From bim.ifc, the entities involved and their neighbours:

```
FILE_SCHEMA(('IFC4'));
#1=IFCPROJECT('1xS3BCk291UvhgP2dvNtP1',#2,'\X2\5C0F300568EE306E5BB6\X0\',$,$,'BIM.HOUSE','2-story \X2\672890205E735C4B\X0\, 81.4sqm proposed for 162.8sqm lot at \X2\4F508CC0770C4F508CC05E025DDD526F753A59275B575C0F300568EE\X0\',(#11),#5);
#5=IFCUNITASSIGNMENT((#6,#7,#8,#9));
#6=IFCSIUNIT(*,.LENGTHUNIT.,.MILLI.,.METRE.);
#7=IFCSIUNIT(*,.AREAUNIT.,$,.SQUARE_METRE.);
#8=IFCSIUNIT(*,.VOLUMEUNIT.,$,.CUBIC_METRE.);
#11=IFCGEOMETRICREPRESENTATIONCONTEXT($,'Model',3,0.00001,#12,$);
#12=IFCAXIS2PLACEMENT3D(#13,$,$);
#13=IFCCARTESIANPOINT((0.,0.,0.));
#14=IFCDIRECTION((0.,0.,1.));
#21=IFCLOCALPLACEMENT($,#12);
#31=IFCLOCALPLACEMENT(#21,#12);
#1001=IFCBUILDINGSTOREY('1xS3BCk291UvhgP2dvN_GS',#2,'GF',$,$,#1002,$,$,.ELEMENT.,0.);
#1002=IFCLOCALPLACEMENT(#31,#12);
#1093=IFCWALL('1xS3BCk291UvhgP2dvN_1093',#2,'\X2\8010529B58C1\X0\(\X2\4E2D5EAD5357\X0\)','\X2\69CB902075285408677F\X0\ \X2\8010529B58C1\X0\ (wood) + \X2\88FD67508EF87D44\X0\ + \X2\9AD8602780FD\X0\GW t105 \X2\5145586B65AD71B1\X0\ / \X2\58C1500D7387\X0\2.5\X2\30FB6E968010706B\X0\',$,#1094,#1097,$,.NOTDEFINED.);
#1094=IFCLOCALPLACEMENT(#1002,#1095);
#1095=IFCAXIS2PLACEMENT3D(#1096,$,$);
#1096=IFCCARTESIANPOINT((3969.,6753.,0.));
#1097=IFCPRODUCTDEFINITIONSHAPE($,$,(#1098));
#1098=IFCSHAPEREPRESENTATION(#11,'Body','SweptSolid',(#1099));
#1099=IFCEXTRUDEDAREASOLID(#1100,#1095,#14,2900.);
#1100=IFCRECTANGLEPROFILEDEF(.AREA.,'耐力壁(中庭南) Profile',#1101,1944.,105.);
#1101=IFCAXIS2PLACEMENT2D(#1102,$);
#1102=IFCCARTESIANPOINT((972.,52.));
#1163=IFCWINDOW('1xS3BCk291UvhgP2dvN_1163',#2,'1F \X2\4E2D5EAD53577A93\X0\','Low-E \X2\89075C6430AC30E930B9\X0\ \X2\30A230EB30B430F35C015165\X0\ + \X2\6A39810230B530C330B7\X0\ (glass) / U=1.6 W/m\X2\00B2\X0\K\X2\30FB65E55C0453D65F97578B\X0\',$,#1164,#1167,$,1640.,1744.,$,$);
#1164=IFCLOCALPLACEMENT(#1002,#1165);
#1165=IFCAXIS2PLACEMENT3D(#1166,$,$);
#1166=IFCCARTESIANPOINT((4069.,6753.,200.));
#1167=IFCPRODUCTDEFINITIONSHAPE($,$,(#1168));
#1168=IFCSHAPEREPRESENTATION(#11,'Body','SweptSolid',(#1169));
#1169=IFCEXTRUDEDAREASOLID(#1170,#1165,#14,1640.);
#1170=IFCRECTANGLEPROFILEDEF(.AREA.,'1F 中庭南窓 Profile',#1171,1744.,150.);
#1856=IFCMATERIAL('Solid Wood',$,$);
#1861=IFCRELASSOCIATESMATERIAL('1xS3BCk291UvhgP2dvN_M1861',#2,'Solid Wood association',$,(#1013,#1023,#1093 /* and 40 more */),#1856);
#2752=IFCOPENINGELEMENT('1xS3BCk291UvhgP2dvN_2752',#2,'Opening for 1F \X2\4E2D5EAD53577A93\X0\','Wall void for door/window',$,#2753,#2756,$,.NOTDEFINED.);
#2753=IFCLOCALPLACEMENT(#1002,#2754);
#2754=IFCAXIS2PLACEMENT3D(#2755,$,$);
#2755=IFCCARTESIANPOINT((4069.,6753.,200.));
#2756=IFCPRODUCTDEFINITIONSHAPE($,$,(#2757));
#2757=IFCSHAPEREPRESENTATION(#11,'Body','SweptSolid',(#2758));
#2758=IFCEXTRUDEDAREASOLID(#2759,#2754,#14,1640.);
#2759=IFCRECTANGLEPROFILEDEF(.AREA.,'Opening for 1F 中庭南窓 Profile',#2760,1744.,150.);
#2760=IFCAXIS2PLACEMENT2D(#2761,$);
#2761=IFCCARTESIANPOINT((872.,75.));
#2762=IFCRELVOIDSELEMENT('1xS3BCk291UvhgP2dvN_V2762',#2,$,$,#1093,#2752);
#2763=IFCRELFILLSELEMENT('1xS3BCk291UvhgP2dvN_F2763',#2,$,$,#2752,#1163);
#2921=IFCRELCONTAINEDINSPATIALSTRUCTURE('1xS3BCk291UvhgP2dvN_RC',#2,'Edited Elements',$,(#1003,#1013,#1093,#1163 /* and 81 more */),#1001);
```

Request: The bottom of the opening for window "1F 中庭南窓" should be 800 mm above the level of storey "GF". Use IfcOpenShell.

```python
import numpy as np
import ifcopenshell
import ifcopenshell.api.geometry
import ifcopenshell.geom
import ifcopenshell.util.element
import ifcopenshell.util.placement
import ifcopenshell.util.shape
import ifcopenshell.util.unit

model = ifcopenshell.open("bim.ifc")
unit_scale = ifcopenshell.util.unit.calculate_unit_scale(model)

window = model.by_guid("1xS3BCk291UvhgP2dvN_1163")
opening = window.FillsVoids[0].RelatingOpeningElement
storey = ifcopenshell.util.element.get_container(window, ifc_class="IfcBuildingStorey")
level = ifcopenshell.util.placement.get_local_placement(storey.ObjectPlacement)[2, 3]

# The opening's origin need not be at the sill, so measure its lowest point.
shape = ifcopenshell.geom.create_shape(ifcopenshell.geom.settings(), opening)
bottom = ifcopenshell.util.shape.get_shape_bottom_elevation(shape, shape.geometry) / unit_scale
dz = level + 800.0 - bottom

shift = np.array([0.0, 0.0, dz])
# The window is not placed relative to its opening, so move both.
for product in (opening, window):
    matrix = ifcopenshell.util.placement.get_local_placement(product.ObjectPlacement)
    matrix[:3, 3] += shift
    ifcopenshell.api.geometry.edit_object_placement(model, product=product, matrix=matrix, is_si=False)

print(f"moved by {dz * unit_scale:+.3f} m")

model.write("bim_v2.ifc")
```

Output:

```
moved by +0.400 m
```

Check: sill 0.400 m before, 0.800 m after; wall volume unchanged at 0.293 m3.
